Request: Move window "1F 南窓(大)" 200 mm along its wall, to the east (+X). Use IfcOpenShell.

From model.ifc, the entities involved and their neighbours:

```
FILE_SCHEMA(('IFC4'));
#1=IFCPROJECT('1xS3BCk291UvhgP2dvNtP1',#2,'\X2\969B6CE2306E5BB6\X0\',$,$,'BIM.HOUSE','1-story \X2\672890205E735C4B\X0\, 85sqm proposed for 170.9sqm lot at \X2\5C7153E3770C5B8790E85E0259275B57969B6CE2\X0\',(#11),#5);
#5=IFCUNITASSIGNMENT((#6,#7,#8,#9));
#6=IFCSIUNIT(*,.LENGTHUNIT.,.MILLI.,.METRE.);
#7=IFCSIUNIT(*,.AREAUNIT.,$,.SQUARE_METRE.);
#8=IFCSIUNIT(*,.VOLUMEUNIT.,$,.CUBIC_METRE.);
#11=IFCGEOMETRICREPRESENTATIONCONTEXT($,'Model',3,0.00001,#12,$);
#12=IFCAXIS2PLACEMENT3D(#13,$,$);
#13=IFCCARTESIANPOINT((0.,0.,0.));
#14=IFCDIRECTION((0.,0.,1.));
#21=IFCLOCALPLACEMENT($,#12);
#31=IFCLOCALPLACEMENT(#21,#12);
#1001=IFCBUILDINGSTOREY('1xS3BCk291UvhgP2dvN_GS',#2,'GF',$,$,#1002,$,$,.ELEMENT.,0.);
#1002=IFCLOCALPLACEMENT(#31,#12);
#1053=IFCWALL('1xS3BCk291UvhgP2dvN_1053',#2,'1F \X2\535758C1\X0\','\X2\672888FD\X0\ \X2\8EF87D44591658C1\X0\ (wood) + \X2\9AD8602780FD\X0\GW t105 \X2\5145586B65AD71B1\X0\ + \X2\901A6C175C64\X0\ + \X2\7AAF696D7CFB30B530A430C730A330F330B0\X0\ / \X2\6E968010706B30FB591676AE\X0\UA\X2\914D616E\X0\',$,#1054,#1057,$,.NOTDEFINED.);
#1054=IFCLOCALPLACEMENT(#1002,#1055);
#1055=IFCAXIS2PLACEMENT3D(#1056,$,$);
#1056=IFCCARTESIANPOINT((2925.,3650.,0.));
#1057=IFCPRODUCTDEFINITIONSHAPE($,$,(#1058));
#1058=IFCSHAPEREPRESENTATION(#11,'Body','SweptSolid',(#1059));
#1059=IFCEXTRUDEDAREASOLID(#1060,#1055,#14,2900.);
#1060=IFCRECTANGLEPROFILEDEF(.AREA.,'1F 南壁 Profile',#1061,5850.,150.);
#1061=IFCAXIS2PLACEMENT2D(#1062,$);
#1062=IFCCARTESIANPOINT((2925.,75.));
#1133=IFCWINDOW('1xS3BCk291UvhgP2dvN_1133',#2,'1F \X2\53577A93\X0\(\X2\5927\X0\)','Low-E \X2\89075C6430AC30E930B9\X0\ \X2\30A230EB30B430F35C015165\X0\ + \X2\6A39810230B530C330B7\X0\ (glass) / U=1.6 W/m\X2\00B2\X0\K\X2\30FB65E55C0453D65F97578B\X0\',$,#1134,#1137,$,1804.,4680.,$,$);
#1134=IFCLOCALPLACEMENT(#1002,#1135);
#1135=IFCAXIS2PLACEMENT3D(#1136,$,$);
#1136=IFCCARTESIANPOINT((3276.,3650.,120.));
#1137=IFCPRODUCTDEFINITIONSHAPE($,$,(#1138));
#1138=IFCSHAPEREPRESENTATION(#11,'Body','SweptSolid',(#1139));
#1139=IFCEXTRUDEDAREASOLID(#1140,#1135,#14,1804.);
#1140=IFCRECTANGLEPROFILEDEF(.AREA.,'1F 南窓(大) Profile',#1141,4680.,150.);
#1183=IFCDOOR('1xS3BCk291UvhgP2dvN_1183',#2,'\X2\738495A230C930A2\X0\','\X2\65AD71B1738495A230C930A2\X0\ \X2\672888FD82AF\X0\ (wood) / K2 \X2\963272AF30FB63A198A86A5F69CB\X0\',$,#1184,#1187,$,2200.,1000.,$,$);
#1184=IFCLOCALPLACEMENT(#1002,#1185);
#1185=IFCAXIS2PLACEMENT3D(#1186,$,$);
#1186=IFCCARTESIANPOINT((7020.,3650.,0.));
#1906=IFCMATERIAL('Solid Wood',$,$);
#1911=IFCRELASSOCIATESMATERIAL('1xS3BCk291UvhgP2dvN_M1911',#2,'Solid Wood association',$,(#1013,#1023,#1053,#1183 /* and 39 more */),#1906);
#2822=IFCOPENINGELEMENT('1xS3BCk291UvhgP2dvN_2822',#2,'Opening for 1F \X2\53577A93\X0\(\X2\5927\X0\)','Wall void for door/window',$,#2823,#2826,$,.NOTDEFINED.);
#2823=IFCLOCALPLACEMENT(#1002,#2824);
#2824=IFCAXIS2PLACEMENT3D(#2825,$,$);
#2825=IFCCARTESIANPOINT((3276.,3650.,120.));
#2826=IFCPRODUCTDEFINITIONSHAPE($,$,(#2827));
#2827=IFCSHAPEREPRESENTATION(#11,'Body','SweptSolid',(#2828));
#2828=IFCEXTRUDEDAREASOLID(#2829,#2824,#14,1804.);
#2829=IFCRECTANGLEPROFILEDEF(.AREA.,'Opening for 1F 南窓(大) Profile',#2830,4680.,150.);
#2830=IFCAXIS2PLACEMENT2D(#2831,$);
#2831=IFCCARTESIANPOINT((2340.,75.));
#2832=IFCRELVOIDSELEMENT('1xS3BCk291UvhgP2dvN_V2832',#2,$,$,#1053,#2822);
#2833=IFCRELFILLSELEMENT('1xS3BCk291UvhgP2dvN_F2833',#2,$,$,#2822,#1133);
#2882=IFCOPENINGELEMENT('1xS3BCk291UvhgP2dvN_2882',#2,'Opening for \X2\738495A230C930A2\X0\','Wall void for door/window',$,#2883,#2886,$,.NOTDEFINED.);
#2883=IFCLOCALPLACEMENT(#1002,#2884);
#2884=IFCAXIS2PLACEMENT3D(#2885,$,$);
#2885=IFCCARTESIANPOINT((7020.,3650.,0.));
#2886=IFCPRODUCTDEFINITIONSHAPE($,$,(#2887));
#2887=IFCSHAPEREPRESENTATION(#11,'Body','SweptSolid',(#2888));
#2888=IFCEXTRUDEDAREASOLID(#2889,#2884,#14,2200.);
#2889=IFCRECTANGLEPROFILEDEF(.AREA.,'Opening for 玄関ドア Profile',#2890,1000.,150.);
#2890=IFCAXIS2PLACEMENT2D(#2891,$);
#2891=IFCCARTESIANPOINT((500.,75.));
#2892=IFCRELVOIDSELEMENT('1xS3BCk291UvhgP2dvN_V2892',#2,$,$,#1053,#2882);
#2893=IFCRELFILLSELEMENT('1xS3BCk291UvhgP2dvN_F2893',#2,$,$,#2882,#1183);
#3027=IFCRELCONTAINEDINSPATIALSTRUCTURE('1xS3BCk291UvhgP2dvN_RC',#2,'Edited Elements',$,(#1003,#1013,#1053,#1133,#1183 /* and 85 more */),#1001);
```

```python
import ifcopenshell
import ifcopenshell.api.geometry
import ifcopenshell.util.placement

model = ifcopenshell.open("model.ifc")

window = model.by_guid("1xS3BCk291UvhgP2dvN_1133")
opening = window.FillsVoids[0].RelatingOpeningElement
wall = opening.VoidsElements[0].RelatingBuildingElement

wall_matrix = ifcopenshell.util.placement.get_local_placement(wall.ObjectPlacement)
shift = wall_matrix[:3, 0] * 200.0
before = ifcopenshell.util.placement.get_local_placement(window.ObjectPlacement)[:3, 3].copy()

# The window is not placed relative to its opening, so move both.
for product in (opening, window):
    matrix = ifcopenshell.util.placement.get_local_placement(product.ObjectPlacement)
    matrix[:3, 3] += shift
    ifcopenshell.api.geometry.edit_object_placement(model, product=product, matrix=matrix, is_si=False)

after = ifcopenshell.util.placement.get_local_placement(window.ObjectPlacement)[:3, 3]
print("window moved by", (after - before).round(3) + 0.0)

model.write("model_rev.ifc")
```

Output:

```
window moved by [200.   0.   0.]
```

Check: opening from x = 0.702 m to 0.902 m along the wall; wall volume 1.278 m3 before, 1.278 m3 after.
